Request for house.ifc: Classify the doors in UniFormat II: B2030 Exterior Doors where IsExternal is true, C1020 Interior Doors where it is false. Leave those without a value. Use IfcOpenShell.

First a look at what the model holds.

```python
import ifcopenshell
import ifcopenshell.util.element

model = ifcopenshell.open("house.ifc")
print(model.schema)
print("classifications:", [c.Name for c in model.by_type("IfcClassification")])
values = [ifcopenshell.util.element.get_pset(e, "Pset_DoorCommon", "IsExternal") for e in model.by_type("IfcDoor")]
for value in (True, False, None):
    print("IsExternal", value, values.count(value))
```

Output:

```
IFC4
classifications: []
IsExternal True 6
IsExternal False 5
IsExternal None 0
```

```python
import ifcopenshell
import ifcopenshell.api.classification
import ifcopenshell.util.element

model = ifcopenshell.open("house.ifc")

system = ifcopenshell.api.classification.add_classification(model, classification="UniFormat II")

doors = model.by_type("IfcDoor")
external = {e: ifcopenshell.util.element.get_pset(e, "Pset_DoorCommon", "IsExternal") for e in doors}
for flag, code, name in ((True, "B2030", "Exterior Doors"), (False, "C1020", "Interior Doors")):
    products = [e for e in doors if external[e] is flag]
    ifcopenshell.api.classification.add_reference(
        model, products=products, classification=system, identification=code, name=name
    )
    print(code, len(products))

model.write("house_rev.ifc")
```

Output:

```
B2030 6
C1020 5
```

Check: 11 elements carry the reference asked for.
